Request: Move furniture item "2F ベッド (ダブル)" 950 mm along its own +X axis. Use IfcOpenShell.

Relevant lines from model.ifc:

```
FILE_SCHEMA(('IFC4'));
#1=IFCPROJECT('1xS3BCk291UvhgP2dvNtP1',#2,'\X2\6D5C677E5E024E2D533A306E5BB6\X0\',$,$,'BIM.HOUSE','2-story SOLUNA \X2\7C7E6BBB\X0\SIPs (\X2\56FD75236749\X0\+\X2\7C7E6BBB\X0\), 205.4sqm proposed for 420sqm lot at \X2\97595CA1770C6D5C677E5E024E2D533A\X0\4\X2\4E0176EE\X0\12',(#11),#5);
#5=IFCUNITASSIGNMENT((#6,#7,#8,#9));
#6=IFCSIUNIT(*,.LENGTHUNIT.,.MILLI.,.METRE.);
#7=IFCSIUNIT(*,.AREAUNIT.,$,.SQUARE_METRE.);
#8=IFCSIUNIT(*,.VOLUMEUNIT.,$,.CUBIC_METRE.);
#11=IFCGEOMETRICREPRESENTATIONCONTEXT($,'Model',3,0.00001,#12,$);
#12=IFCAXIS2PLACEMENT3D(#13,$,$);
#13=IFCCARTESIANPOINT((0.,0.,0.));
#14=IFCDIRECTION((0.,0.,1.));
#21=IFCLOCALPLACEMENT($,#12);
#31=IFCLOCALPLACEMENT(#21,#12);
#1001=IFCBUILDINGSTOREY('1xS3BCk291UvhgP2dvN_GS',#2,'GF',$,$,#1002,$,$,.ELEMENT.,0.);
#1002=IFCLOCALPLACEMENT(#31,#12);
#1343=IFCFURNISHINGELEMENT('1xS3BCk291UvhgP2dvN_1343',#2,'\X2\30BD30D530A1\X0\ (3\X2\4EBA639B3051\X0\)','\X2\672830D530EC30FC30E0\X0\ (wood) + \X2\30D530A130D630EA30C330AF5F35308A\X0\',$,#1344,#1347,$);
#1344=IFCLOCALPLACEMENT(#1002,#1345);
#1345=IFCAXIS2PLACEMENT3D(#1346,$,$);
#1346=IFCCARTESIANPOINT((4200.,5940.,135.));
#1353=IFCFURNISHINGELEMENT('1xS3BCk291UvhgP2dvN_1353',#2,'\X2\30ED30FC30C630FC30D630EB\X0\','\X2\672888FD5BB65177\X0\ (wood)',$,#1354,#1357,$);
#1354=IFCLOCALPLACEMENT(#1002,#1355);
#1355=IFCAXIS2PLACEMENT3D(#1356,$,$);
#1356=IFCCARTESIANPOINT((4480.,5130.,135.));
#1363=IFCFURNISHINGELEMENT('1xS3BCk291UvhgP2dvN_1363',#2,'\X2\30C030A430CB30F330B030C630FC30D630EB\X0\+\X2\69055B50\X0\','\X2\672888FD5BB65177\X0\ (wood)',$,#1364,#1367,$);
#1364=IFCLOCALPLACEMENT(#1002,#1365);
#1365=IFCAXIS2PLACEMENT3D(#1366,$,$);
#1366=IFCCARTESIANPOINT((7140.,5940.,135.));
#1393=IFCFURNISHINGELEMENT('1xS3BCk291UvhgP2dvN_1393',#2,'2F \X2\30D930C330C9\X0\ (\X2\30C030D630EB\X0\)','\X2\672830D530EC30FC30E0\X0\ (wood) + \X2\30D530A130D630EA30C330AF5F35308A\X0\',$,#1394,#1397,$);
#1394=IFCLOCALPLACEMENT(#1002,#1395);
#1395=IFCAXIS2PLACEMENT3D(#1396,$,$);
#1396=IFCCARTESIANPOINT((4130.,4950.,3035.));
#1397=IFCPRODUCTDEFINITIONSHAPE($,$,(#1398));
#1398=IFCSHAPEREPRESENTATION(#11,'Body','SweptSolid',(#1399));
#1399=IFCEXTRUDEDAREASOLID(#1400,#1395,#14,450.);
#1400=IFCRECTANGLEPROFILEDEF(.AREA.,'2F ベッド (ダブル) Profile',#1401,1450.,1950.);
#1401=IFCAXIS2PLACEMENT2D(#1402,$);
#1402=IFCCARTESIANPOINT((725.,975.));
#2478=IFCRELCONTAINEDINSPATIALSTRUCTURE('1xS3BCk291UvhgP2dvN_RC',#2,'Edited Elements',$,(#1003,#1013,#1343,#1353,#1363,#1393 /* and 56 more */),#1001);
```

```python
import ifcopenshell
import ifcopenshell.api.geometry
import ifcopenshell.util.placement

model = ifcopenshell.open("model.ifc")

item = model.by_id(1393)
matrix = ifcopenshell.util.placement.get_local_placement(item.ObjectPlacement)
matrix[:3, 3] += matrix[:3, 0] * 950.0
ifcopenshell.api.geometry.edit_object_placement(model, product=item, matrix=matrix, is_si=False)

print(ifcopenshell.util.placement.get_local_placement(item.ObjectPlacement).round(3) + 0.0)

model.write("model-out.ifc")
```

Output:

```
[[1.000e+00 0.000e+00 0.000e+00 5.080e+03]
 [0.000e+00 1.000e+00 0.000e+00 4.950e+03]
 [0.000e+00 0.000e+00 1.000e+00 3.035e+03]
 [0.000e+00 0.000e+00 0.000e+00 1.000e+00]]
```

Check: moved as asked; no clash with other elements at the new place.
